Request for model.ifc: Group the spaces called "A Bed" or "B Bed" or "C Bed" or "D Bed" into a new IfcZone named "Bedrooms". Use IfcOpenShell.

First a look at what the model holds.

```python
import ifcopenshell

model = ifcopenshell.open("model.ifc")
print(model.schema)
seen = {}
for space in model.by_type("IfcSpace"):
    seen[space.Name] = seen.get(space.Name, 0) + 1
for name, count in sorted(seen.items(), key=str):
    print(count, "x", name)
print("zones:", [z.Name for z in model.by_type("IfcZone")][:20])
```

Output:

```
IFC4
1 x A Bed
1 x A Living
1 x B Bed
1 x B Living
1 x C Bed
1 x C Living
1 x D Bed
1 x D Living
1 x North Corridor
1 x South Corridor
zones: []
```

```python
import ifcopenshell
import ifcopenshell.api.group
import ifcopenshell.api.root

model = ifcopenshell.open("model.ifc")

names = {"A Bed", "B Bed", "C Bed", "D Bed"}
spaces = [s for s in model.by_type("IfcSpace") if s.Name in names]

zone = ifcopenshell.api.root.create_entity(model, ifc_class="IfcZone", name="Bedrooms")
ifcopenshell.api.group.assign_group(model, products=spaces, group=zone)
print(len(spaces), "spaces in", zone.Name)

model.write("model_rev.ifc")
```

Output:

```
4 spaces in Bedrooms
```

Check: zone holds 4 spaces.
